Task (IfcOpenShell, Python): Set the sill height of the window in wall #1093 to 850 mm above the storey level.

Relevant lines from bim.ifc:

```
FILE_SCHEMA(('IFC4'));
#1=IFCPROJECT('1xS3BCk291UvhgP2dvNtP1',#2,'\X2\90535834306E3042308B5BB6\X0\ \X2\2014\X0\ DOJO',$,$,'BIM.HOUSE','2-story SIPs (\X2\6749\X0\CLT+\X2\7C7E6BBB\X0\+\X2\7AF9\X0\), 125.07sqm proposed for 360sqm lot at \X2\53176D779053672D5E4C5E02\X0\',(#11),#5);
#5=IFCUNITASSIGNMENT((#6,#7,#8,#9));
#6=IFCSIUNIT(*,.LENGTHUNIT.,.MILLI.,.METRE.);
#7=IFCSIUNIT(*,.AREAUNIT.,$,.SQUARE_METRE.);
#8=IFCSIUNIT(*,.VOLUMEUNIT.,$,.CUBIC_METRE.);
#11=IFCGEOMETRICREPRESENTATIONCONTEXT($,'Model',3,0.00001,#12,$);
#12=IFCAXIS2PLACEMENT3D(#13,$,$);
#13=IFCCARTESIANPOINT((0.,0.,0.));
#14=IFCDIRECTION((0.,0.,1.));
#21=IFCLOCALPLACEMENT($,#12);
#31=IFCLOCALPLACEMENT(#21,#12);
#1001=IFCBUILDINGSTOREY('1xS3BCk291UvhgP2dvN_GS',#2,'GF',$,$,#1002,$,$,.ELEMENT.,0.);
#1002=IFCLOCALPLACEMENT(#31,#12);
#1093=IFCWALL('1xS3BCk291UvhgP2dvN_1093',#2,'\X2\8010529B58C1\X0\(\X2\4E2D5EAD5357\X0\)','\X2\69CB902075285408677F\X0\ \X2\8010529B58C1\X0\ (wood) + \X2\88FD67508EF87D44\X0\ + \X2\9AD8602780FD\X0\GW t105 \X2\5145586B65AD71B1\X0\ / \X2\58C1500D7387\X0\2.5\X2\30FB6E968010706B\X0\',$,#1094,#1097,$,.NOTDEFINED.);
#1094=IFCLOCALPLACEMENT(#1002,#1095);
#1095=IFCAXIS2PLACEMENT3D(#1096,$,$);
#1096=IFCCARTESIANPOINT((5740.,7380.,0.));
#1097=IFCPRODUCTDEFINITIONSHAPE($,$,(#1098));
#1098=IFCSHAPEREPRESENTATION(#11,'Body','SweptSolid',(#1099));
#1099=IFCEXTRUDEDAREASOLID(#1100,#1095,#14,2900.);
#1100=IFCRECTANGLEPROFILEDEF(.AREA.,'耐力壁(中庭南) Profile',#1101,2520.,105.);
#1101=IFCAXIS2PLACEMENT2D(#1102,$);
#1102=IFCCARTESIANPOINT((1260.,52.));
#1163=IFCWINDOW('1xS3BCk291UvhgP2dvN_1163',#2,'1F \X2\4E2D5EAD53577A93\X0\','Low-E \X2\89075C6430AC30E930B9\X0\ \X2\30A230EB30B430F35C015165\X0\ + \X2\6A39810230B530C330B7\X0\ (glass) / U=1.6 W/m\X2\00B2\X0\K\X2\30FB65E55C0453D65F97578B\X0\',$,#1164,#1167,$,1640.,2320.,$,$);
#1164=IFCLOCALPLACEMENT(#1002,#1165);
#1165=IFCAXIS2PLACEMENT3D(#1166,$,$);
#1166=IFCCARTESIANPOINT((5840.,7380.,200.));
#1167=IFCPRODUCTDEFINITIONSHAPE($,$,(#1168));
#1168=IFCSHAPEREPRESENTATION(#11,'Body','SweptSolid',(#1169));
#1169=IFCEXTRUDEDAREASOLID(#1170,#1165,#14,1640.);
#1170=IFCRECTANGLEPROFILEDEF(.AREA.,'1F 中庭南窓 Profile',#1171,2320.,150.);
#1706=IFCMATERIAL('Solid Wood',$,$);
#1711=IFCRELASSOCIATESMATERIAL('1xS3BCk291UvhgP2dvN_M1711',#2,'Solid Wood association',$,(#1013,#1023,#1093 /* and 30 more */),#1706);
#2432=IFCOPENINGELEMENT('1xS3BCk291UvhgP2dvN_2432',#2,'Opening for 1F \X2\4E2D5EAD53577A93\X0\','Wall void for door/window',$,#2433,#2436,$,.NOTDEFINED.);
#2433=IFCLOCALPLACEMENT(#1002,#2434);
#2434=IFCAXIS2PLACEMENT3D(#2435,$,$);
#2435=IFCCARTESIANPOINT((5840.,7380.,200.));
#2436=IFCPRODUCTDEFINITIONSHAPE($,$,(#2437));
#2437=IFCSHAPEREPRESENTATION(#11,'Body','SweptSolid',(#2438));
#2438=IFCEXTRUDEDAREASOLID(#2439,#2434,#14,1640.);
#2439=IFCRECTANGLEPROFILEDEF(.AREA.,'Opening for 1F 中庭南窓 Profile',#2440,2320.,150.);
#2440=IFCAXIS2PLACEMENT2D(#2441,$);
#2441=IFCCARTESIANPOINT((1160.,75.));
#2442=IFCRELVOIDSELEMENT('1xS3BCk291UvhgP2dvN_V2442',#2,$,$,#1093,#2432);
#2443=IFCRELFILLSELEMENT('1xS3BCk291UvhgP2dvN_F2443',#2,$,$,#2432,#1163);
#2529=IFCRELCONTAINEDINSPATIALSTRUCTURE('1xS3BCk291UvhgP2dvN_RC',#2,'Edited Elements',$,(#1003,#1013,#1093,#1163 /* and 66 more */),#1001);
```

```python
import numpy as np
import ifcopenshell
import ifcopenshell.api.geometry
import ifcopenshell.geom
import ifcopenshell.util.element
import ifcopenshell.util.placement
import ifcopenshell.util.shape
import ifcopenshell.util.unit

model = ifcopenshell.open("bim.ifc")
unit_scale = ifcopenshell.util.unit.calculate_unit_scale(model)

window = model.by_guid("1xS3BCk291UvhgP2dvN_1163")
opening = window.FillsVoids[0].RelatingOpeningElement
storey = ifcopenshell.util.element.get_container(window, ifc_class="IfcBuildingStorey")
level = ifcopenshell.util.placement.get_local_placement(storey.ObjectPlacement)[2, 3]

# The opening's origin need not be at the sill, so measure its lowest point.
shape = ifcopenshell.geom.create_shape(ifcopenshell.geom.settings(), opening)
bottom = ifcopenshell.util.shape.get_shape_bottom_elevation(shape, shape.geometry) / unit_scale
dz = level + 850.0 - bottom

shift = np.array([0.0, 0.0, dz])
# The window is not placed relative to its opening, so move both.
for product in (opening, window):
    matrix = ifcopenshell.util.placement.get_local_placement(product.ObjectPlacement)
    matrix[:3, 3] += shift
    ifcopenshell.api.geometry.edit_object_placement(model, product=product, matrix=matrix, is_si=False)

print(f"moved by {dz * unit_scale:+.3f} m")

model.write("bim_v2.ifc")
```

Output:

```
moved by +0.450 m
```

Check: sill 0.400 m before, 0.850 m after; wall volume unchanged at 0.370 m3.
